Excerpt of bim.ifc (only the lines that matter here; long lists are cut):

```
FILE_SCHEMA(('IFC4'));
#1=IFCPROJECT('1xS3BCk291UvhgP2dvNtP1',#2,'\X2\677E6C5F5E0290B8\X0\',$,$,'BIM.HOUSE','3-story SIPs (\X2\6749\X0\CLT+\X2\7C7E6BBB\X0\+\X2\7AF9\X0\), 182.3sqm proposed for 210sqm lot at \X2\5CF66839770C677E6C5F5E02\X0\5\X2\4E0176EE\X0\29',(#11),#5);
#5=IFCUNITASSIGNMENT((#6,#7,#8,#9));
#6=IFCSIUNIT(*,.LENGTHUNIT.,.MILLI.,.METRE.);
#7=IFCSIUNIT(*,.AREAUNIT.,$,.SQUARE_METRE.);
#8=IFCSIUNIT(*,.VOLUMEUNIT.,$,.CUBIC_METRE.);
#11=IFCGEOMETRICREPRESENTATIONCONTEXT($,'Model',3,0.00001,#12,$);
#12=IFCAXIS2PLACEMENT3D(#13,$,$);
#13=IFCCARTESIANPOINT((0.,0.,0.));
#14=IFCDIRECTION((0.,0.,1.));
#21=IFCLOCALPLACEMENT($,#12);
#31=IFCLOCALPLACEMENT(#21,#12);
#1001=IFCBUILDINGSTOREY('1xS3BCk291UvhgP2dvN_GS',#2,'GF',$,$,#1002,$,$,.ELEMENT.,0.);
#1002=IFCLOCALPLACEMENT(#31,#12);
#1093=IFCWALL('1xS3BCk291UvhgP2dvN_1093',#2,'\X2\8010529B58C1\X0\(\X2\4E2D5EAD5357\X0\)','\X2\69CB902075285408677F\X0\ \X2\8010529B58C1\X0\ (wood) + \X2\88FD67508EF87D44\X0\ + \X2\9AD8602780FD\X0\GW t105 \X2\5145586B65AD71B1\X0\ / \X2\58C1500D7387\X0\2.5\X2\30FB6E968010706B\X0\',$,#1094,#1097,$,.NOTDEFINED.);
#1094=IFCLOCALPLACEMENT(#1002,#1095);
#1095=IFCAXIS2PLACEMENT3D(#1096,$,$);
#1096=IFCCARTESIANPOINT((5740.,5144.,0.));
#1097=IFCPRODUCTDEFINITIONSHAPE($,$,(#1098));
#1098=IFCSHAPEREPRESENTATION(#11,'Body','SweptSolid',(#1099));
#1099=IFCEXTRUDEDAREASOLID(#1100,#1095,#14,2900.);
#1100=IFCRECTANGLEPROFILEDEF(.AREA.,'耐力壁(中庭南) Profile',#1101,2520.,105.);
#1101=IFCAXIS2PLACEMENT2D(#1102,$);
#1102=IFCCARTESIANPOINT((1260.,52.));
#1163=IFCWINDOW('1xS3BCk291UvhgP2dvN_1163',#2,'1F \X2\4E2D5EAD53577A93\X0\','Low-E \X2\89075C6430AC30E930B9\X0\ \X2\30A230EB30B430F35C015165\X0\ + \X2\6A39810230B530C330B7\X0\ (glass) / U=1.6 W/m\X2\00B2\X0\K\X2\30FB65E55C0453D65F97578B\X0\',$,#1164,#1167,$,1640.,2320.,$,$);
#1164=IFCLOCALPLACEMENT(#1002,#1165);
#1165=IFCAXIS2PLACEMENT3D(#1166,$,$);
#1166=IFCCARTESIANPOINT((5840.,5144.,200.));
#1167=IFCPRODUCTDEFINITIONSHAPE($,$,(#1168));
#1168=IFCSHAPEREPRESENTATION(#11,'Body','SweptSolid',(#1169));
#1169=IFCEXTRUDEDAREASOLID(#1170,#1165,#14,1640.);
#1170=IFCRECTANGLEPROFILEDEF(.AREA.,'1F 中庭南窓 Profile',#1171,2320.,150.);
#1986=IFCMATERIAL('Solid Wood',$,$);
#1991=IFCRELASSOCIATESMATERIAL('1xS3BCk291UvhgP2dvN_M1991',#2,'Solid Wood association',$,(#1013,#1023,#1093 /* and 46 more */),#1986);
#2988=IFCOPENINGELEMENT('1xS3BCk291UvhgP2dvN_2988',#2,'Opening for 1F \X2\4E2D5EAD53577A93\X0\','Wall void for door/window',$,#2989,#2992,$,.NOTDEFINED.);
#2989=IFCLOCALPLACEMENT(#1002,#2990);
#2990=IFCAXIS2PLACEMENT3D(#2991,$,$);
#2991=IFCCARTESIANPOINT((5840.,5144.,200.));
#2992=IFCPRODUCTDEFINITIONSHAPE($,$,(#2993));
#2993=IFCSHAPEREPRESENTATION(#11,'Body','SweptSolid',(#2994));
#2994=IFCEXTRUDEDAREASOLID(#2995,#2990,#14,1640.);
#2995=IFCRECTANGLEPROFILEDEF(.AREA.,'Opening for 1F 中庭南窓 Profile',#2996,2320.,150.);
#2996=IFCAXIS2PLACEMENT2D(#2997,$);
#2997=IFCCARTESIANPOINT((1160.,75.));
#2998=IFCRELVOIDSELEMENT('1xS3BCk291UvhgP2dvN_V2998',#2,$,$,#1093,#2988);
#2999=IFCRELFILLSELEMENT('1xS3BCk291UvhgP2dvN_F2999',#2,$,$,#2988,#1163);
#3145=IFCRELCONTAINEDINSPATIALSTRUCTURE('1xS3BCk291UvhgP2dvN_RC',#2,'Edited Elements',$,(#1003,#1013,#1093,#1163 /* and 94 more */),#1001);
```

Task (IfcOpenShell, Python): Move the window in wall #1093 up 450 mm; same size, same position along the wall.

```python
import numpy as np
import ifcopenshell
import ifcopenshell.api.geometry
import ifcopenshell.util.placement
import ifcopenshell.util.unit

model = ifcopenshell.open("bim.ifc")
unit_scale = ifcopenshell.util.unit.calculate_unit_scale(model)

window = model.by_guid("1xS3BCk291UvhgP2dvN_1163")
opening = window.FillsVoids[0].RelatingOpeningElement
dz = 450.0

shift = np.array([0.0, 0.0, dz])
# The window is not placed relative to its opening, so move both.
for product in (opening, window):
    matrix = ifcopenshell.util.placement.get_local_placement(product.ObjectPlacement)
    matrix[:3, 3] += shift
    ifcopenshell.api.geometry.edit_object_placement(model, product=product, matrix=matrix, is_si=False)

print(f"moved by {dz * unit_scale:+.3f} m")

model.write("bim_v2.ifc")
```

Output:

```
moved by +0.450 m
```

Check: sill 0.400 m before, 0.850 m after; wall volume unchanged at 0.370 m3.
